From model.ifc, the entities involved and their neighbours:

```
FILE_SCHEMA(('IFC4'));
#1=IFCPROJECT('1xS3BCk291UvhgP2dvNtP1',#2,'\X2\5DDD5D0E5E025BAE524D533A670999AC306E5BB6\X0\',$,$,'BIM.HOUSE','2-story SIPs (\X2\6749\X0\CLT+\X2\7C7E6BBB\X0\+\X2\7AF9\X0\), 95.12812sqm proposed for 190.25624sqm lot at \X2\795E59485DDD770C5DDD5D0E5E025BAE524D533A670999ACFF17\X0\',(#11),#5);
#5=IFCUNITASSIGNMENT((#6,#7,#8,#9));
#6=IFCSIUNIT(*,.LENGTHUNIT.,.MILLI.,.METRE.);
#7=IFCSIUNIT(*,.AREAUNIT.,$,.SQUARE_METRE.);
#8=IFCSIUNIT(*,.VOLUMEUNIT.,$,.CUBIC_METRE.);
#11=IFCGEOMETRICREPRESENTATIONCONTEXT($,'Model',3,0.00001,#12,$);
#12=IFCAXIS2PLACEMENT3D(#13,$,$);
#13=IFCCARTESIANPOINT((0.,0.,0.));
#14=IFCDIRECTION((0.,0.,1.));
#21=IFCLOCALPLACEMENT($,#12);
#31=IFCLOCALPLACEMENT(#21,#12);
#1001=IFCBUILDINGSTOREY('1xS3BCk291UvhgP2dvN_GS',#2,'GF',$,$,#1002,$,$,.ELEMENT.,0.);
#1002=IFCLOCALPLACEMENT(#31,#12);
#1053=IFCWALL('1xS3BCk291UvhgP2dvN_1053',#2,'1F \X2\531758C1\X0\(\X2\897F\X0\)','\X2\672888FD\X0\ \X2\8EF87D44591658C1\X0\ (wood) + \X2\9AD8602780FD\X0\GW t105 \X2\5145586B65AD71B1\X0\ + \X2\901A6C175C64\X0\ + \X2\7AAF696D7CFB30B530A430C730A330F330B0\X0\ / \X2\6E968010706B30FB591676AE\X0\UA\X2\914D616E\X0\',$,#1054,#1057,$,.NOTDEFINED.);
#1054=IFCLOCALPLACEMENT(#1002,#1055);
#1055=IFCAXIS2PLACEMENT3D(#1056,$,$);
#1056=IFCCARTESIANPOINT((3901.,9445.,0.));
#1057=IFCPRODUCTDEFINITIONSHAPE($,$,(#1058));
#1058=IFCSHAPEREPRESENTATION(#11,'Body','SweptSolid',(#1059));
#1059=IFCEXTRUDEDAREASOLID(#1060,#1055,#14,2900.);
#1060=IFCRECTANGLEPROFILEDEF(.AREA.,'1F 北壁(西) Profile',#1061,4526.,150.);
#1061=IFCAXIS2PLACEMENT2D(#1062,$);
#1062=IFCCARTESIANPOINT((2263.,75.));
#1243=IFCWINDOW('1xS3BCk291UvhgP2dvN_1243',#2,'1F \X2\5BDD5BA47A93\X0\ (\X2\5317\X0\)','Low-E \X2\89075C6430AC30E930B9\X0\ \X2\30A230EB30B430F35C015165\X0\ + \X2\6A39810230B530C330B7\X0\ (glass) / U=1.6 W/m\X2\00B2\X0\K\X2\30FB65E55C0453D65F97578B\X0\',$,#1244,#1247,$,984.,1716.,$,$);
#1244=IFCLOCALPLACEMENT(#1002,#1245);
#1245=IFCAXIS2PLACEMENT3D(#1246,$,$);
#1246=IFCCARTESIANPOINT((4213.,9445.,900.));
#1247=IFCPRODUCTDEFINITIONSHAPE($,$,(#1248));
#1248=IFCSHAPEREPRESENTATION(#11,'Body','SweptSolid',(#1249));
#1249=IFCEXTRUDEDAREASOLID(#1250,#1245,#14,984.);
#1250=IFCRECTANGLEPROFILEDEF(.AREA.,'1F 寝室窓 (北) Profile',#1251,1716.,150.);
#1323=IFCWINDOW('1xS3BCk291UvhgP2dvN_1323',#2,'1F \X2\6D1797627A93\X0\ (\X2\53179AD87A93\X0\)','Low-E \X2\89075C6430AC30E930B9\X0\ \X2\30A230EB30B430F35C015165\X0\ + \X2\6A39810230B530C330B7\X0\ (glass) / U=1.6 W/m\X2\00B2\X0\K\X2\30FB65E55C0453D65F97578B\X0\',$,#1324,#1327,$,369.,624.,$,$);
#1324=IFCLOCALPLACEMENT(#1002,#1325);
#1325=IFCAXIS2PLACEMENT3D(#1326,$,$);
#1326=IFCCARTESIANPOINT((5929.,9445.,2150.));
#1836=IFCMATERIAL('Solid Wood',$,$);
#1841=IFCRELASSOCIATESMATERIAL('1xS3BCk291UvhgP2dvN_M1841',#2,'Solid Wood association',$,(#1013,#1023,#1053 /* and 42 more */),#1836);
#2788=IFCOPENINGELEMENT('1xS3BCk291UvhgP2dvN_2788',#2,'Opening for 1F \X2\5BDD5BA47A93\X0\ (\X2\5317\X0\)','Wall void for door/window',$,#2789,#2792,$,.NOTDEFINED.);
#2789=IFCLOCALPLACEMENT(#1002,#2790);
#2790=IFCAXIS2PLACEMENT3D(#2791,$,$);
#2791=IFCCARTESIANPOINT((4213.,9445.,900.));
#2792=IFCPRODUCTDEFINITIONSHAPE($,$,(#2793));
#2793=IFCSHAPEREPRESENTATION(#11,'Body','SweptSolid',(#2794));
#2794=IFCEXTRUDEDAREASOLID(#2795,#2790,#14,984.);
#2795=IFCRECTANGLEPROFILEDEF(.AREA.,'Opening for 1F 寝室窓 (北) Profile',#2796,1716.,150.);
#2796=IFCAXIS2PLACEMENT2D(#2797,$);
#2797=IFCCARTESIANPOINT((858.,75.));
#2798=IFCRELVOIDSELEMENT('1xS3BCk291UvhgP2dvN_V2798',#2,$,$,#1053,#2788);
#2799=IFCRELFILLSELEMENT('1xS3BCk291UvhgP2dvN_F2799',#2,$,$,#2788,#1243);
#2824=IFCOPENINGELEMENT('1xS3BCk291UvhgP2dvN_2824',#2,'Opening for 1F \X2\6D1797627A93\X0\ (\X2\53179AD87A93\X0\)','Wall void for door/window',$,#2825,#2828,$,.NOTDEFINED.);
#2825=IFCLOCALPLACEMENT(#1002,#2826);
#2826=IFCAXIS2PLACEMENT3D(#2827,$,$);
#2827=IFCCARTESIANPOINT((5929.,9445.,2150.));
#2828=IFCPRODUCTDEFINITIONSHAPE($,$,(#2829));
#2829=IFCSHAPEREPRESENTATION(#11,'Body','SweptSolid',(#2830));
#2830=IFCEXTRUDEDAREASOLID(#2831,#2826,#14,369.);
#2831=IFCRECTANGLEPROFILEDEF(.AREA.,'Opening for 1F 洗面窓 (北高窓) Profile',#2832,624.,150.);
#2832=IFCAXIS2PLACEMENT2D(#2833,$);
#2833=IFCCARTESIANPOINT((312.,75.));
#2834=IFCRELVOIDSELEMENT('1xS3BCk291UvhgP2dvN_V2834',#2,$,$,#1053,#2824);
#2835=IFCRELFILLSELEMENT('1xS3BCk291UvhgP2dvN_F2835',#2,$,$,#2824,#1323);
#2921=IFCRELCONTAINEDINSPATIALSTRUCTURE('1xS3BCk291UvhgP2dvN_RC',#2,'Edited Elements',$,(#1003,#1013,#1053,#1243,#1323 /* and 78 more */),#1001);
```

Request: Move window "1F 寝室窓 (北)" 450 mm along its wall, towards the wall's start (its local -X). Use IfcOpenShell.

```python
import ifcopenshell
import ifcopenshell.api.geometry
import ifcopenshell.util.placement
import ifcopenshell.util.unit

model = ifcopenshell.open("model.ifc")
unit_scale = ifcopenshell.util.unit.calculate_unit_scale(model)

window = model.by_guid("1xS3BCk291UvhgP2dvN_1243")
opening = window.FillsVoids[0].RelatingOpeningElement
wall = opening.VoidsElements[0].RelatingBuildingElement

wall_matrix = ifcopenshell.util.placement.get_local_placement(wall.ObjectPlacement)
shift = wall_matrix[:3, 0] * -0.45 / unit_scale
before = ifcopenshell.util.placement.get_local_placement(window.ObjectPlacement)[:3, 3].copy()

# The window is not placed relative to its opening, so move both.
for product in (opening, window):
    matrix = ifcopenshell.util.placement.get_local_placement(product.ObjectPlacement)
    matrix[:3, 3] += shift
    ifcopenshell.api.geometry.edit_object_placement(model, product=product, matrix=matrix, is_si=False)

after = ifcopenshell.util.placement.get_local_placement(window.ObjectPlacement)[:3, 3]
print("window moved by", (after - before).round(3) + 0.0)

model.write("model_v2.ifc")
```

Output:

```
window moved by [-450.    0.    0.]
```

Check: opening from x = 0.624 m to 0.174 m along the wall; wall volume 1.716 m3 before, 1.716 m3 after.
